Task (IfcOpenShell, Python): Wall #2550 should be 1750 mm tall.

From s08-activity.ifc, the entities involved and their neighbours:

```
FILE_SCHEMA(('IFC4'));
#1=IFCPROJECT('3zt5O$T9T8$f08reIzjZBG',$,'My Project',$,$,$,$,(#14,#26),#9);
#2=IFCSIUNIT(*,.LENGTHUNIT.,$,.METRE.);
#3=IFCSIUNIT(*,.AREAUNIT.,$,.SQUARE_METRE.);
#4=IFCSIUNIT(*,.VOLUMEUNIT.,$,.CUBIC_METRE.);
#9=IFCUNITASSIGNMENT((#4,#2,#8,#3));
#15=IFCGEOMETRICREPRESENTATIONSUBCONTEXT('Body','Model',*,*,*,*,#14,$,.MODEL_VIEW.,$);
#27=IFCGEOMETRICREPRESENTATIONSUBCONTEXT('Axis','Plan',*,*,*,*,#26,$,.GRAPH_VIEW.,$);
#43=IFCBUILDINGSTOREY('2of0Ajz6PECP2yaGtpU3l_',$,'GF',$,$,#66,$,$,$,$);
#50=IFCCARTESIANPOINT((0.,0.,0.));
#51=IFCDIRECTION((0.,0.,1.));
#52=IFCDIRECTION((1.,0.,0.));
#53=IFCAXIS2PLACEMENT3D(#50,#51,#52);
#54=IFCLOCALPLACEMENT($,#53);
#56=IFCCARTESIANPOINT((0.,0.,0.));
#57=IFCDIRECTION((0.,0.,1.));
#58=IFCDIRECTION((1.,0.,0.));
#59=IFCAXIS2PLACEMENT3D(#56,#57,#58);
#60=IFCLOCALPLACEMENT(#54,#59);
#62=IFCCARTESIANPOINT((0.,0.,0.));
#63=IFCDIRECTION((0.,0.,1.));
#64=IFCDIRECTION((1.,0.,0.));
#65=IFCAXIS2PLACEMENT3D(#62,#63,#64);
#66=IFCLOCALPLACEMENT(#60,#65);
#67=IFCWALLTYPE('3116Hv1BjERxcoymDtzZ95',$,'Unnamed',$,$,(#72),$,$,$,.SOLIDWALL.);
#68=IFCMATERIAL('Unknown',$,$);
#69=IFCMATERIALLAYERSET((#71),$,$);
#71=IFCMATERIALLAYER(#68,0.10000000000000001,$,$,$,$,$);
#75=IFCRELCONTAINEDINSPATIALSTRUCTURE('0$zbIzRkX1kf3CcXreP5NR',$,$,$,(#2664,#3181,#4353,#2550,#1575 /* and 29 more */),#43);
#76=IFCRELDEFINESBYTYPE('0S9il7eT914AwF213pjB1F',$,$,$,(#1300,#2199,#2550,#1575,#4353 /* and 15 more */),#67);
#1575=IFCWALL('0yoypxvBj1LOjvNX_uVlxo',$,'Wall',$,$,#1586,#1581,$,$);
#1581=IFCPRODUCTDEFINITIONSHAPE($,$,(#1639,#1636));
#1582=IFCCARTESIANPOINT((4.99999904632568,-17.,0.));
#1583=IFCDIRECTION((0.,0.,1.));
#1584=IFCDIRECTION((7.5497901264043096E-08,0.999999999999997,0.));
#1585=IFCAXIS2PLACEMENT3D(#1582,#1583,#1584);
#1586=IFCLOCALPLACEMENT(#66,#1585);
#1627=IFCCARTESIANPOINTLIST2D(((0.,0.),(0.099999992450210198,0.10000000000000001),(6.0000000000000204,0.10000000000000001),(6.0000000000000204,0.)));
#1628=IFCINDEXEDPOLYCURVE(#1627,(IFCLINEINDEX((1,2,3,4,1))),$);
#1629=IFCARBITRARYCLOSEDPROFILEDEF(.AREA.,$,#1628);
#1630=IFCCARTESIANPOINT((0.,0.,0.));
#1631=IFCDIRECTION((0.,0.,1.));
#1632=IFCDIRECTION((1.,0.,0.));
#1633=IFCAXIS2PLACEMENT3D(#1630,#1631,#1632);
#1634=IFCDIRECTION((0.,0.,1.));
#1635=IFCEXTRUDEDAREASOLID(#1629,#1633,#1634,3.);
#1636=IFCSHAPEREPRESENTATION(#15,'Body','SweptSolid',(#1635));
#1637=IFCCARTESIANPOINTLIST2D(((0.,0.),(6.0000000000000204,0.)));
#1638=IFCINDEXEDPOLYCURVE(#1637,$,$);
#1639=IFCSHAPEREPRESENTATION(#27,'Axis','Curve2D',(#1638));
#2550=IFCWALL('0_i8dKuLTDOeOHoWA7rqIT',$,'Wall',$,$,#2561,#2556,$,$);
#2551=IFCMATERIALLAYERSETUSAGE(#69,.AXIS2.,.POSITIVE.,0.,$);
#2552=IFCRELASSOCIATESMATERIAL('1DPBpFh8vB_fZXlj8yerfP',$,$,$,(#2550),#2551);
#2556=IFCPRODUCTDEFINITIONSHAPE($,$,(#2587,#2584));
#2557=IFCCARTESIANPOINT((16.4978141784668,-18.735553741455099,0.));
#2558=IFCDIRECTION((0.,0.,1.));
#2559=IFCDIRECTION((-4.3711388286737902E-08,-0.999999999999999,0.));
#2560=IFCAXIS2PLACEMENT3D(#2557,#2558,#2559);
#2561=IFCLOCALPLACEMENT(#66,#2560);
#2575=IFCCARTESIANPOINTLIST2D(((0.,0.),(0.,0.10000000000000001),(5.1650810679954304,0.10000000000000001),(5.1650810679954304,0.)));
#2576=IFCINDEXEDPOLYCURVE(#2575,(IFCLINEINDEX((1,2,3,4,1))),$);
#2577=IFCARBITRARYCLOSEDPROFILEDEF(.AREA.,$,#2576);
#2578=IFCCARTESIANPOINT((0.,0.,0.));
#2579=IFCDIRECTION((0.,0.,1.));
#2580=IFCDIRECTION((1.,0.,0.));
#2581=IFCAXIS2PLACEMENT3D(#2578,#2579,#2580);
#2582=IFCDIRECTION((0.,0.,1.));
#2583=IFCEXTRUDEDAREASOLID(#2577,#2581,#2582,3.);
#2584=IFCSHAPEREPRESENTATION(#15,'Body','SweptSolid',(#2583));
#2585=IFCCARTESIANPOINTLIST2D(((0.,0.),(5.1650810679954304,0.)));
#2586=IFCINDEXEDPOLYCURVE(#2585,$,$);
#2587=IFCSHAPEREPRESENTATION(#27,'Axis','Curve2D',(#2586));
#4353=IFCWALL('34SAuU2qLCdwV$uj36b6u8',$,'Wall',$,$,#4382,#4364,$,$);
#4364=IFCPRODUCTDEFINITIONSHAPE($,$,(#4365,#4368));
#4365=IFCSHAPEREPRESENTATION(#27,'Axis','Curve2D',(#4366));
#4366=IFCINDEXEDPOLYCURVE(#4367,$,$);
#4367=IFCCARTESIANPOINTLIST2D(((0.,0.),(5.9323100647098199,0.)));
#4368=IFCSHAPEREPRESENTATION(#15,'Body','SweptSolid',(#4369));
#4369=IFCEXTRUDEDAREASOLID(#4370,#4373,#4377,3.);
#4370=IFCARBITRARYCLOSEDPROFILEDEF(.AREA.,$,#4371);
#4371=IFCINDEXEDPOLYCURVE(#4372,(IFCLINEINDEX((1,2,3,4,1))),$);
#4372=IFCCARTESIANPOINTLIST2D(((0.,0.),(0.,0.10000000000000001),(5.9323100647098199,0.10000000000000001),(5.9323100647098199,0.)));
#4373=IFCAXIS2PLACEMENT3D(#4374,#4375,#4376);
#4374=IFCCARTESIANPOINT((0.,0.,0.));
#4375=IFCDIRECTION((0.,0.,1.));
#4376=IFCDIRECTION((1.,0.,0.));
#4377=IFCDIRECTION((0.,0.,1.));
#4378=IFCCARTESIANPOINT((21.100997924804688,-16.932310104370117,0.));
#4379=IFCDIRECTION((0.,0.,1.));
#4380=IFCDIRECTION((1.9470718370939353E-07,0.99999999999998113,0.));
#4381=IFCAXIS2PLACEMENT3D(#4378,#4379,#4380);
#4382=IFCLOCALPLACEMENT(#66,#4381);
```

```python
import ifcopenshell
import ifcopenshell.geom
import ifcopenshell.util.representation
import ifcopenshell.util.shape

model = ifcopenshell.open("s08-activity.ifc")
settings = ifcopenshell.geom.settings()


def volume(element):
    """Net volume in cubic metres, openings subtracted."""
    shape = ifcopenshell.geom.create_shape(settings, element)
    return ifcopenshell.util.shape.get_volume(shape.geometry)


wall = model.by_guid("0_i8dKuLTDOeOHoWA7rqIT")
before = volume(wall)

body = ifcopenshell.util.representation.get_representation(wall, "Model", "Body")
solid = body.Items[0]
old_height = solid.Depth
solid.Depth = 1.75
after = volume(wall)

print(f"height {old_height:g} -> {solid.Depth:g}, volume {before:.3f} -> {after:.3f} m3")

model.write("s08-activity_rev.ifc")
```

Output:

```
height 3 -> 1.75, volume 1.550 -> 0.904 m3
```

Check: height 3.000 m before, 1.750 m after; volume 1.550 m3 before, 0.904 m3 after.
